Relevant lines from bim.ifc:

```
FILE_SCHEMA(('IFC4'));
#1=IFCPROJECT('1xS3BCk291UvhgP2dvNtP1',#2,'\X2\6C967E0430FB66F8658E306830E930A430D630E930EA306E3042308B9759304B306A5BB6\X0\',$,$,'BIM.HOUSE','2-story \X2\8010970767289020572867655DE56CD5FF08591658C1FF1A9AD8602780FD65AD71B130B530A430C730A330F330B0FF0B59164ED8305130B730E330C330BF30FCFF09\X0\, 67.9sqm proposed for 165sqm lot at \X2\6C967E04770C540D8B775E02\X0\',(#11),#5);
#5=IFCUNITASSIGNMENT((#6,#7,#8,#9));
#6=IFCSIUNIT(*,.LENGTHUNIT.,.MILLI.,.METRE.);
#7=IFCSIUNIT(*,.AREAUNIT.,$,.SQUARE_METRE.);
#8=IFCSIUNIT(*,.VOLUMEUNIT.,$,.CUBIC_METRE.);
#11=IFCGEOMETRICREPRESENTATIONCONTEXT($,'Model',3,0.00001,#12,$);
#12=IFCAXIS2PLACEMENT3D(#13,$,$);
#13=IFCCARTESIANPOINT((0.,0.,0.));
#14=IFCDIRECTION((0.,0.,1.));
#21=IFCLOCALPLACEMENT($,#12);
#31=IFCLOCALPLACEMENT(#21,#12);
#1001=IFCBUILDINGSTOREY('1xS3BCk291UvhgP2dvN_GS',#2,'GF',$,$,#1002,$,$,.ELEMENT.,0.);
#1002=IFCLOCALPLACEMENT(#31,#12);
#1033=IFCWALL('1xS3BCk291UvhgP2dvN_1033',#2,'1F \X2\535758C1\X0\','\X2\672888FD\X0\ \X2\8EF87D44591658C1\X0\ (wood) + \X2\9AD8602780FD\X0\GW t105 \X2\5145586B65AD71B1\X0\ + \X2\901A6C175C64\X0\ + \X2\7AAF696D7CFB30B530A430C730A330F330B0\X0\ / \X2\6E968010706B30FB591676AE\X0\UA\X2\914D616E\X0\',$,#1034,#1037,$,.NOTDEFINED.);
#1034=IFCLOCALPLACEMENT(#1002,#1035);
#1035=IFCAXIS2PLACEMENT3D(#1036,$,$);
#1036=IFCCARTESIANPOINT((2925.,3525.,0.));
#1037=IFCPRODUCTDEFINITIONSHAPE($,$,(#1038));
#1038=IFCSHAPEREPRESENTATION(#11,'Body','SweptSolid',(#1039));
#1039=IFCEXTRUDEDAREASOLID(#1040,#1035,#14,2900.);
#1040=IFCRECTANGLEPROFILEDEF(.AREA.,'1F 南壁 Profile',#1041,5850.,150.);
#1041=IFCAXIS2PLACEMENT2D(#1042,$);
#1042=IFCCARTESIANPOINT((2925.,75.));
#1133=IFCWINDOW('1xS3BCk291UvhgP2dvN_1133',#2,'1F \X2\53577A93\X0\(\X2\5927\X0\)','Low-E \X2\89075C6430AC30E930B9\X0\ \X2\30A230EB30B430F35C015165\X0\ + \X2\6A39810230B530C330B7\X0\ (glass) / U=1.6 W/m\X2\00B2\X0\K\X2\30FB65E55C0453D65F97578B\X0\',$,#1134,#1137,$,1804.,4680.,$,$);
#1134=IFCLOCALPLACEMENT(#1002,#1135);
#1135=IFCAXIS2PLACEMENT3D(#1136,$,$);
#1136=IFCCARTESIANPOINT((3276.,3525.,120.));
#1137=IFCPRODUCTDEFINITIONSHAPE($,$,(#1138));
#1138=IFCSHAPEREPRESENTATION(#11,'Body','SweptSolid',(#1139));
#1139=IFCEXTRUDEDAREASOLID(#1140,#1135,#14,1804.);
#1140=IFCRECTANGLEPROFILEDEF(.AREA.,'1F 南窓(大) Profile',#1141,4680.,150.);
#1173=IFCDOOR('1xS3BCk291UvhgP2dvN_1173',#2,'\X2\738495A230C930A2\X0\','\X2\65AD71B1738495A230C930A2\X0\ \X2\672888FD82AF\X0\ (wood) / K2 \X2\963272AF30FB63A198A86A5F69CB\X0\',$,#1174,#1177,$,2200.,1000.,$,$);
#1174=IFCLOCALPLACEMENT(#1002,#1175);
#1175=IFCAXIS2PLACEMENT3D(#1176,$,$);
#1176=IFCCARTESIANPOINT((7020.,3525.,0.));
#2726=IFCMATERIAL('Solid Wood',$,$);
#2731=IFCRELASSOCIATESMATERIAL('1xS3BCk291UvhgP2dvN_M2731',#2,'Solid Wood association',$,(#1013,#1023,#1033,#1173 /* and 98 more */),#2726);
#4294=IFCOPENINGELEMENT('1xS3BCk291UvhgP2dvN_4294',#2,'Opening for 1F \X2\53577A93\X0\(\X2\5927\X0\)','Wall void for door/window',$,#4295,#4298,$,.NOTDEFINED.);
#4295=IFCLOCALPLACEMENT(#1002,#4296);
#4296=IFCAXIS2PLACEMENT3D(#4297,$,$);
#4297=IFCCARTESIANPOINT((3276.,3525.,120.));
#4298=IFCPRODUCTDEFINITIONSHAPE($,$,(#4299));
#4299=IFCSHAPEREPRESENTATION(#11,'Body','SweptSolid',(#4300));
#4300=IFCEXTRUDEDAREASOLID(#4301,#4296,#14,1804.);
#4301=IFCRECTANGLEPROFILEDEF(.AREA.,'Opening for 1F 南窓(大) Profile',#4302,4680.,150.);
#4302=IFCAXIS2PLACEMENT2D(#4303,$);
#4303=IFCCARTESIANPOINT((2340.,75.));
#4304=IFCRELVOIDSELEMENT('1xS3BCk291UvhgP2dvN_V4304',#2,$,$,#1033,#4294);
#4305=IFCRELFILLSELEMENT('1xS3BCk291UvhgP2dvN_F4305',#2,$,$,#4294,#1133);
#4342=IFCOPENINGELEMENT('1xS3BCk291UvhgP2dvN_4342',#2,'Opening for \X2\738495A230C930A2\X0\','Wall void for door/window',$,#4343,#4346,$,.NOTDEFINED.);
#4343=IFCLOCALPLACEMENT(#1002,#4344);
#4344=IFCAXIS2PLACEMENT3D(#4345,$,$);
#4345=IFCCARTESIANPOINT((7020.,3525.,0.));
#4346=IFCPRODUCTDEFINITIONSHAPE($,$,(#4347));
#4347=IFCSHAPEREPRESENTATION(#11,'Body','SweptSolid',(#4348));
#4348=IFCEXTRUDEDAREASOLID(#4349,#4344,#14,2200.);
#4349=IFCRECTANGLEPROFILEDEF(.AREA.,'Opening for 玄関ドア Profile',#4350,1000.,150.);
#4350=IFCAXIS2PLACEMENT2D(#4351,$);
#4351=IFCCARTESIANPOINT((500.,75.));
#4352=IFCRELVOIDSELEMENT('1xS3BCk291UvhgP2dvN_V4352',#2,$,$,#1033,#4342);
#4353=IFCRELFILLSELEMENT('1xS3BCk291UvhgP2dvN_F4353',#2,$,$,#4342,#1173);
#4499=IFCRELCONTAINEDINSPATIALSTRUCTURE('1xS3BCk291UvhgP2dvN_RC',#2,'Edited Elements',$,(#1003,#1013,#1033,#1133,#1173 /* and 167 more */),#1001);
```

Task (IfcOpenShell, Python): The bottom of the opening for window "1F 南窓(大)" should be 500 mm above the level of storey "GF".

```python
import numpy as np
import ifcopenshell
import ifcopenshell.api.geometry
import ifcopenshell.geom
import ifcopenshell.util.element
import ifcopenshell.util.placement
import ifcopenshell.util.shape
import ifcopenshell.util.unit

model = ifcopenshell.open("bim.ifc")
unit_scale = ifcopenshell.util.unit.calculate_unit_scale(model)

window = model.by_guid("1xS3BCk291UvhgP2dvN_1133")
opening = window.FillsVoids[0].RelatingOpeningElement
storey = ifcopenshell.util.element.get_container(window, ifc_class="IfcBuildingStorey")
level = ifcopenshell.util.placement.get_local_placement(storey.ObjectPlacement)[2, 3]

# The opening's origin need not be at the sill, so measure its lowest point.
shape = ifcopenshell.geom.create_shape(ifcopenshell.geom.settings(), opening)
bottom = ifcopenshell.util.shape.get_shape_bottom_elevation(shape, shape.geometry) / unit_scale
dz = level + 0.5 / unit_scale - bottom

shift = np.array([0.0, 0.0, dz])
# The window is not placed relative to its opening, so move both.
for product in (opening, window):
    matrix = ifcopenshell.util.placement.get_local_placement(product.ObjectPlacement)
    matrix[:3, 3] += shift
    ifcopenshell.api.geometry.edit_object_placement(model, product=product, matrix=matrix, is_si=False)

print(f"moved by {dz * unit_scale:+.3f} m")

model.write("bim_v2.ifc")
```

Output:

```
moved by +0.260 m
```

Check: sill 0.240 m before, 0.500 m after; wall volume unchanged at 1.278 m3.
